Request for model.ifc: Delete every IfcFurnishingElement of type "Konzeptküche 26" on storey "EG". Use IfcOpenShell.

First a look at what the model holds.

```python
import ifcopenshell
import ifcopenshell.util.element

model = ifcopenshell.open("model.ifc")
print(model.schema)
storey = next(s for s in model.by_type("IfcBuildingStorey") if s.Name == "EG")
furniture = [e for e in ifcopenshell.util.element.get_decomposition(storey) if e.is_a("IfcFurnishingElement")]
seen = {}
for e in furniture:
    element_type = ifcopenshell.util.element.get_type(e)
    name = element_type.Name if element_type not in (None, e) else None
    seen[name] = seen.get(name, 0) + 1
for name, count in sorted(seen.items(), key=str):
    print(count, "x", name)
```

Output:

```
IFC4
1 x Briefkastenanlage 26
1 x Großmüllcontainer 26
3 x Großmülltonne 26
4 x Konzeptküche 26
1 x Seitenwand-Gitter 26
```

```python
import ifcopenshell
import ifcopenshell.api.root
import ifcopenshell.util.element

model = ifcopenshell.open("model.ifc")

storey = next(s for s in model.by_type("IfcBuildingStorey") if s.Name == "EG")
furniture = [e for e in ifcopenshell.util.element.get_decomposition(storey) if e.is_a("IfcFurnishingElement")]
targets = [e for e in furniture if (t := ifcopenshell.util.element.get_type(e)) not in (None, e) and t.Name == "Konzeptküche 26"]

for e in targets:
    ifcopenshell.api.root.remove_product(model, product=e)
print(len(targets), "removed")

model.write("model-out.ifc")
```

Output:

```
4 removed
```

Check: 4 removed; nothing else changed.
